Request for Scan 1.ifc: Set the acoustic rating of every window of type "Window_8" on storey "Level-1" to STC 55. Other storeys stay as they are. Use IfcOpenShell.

First a look at what the model holds.

```python
import ifcopenshell
import ifcopenshell.util.element

model = ifcopenshell.open("Scan 1.ifc")
print(model.schema)
storey = next(s for s in model.by_type("IfcBuildingStorey") if s.Name == "Level-1")
windows = [e for e in ifcopenshell.util.element.get_decomposition(storey) if e.is_a("IfcWindow")]
seen = {}
for e in windows:
    element_type = ifcopenshell.util.element.get_type(e)
    key = (element_type.Name if element_type != e and element_type else None, ifcopenshell.util.element.get_pset(e, "Pset_WindowCommon", "AcousticRating"))
    seen[key] = seen.get(key, 0) + 1
for (name, value), count in sorted(seen.items(), key=str):
    print(count, "x", name, "|", value)
```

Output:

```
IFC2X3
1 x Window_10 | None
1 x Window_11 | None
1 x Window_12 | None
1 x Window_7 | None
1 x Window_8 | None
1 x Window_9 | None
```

```python
import ifcopenshell
import ifcopenshell.api.pset
import ifcopenshell.util.element

model = ifcopenshell.open("Scan 1.ifc")

storey = next(s for s in model.by_type("IfcBuildingStorey") if s.Name == "Level-1")
windows = [e for e in ifcopenshell.util.element.get_decomposition(storey) if e.is_a("IfcWindow")]

count = 0
for e in windows:
    element_type = ifcopenshell.util.element.get_type(e)
    if element_type in (None, e) or element_type.Name != "Window_8":
        continue
    # add_pset returns the element's existing set when there is one.
    pset = ifcopenshell.api.pset.add_pset(model, product=e, name="Pset_WindowCommon")
    ifcopenshell.api.pset.edit_pset(model, pset=pset, properties={"AcousticRating": "STC 55"})
    count += 1

print(count, "windows updated")

model.write("Scan 1_v2.ifc")
```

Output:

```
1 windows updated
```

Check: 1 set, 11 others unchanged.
